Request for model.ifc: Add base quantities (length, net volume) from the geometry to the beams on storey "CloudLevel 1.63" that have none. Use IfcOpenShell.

First a look at what the model holds.

```python
import ifcopenshell
import ifcopenshell.util.element
import ifcopenshell.util.unit

model = ifcopenshell.open("model.ifc")
print(model.schema)
for unit_type in ("LENGTHUNIT", "AREAUNIT", "VOLUMEUNIT"):
    print(unit_type, ifcopenshell.util.unit.calculate_unit_scale(model, unit_type))
storey = next(s for s in model.by_type("IfcBuildingStorey") if s.Name == "CloudLevel 1.63")
beams = [e for e in ifcopenshell.util.element.get_decomposition(storey) if e.is_a("IfcBeam")]
for e in sorted(beams, key=lambda e: e.id()):
    print(e.id(), e.is_a(), e.Name, list(ifcopenshell.util.element.get_psets(e, qtos_only=True)), sep=" | ")
```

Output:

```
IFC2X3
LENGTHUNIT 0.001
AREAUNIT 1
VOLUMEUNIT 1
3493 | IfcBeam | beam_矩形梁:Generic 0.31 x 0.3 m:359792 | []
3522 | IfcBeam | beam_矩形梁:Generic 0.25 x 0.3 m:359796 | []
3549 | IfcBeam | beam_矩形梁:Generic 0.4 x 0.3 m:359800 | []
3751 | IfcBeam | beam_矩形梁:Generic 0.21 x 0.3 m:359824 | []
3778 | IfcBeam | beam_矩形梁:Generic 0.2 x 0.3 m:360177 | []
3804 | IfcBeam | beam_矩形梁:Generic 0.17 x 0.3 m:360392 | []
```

```python
import ifcopenshell
import ifcopenshell.api.pset
import ifcopenshell.geom
import ifcopenshell.util.element
import ifcopenshell.util.shape
import ifcopenshell.util.unit

model = ifcopenshell.open("model.ifc")
unit_scale = ifcopenshell.util.unit.calculate_unit_scale(model)
volume_scale = ifcopenshell.util.unit.calculate_unit_scale(model, "VOLUMEUNIT")
settings = ifcopenshell.geom.settings()

storey = next(s for s in model.by_type("IfcBuildingStorey") if s.Name == "CloudLevel 1.63")
beams = [e for e in ifcopenshell.util.element.get_decomposition(storey) if e.is_a("IfcBeam")]

for e in sorted(beams, key=lambda e: e.id()):
    if ifcopenshell.util.element.get_psets(e, qtos_only=True, should_inherit=False):
        continue
    # Geometry comes back in metres, in the element's own axes.
    shape = ifcopenshell.geom.create_shape(settings, e)
    values = {
        "Length": ifcopenshell.util.shape.get_max_xyz(shape.geometry) / unit_scale,
        "NetVolume": ifcopenshell.util.shape.get_volume(shape.geometry) / volume_scale,
    }
    qto = ifcopenshell.api.pset.add_qto(model, product=e, name="BaseQuantities")
    ifcopenshell.api.pset.edit_qto(model, qto=qto, properties=values)
    print(e.id(), {k: round(v, 3) for k, v in values.items()})

model.write("model_updated.ifc")
```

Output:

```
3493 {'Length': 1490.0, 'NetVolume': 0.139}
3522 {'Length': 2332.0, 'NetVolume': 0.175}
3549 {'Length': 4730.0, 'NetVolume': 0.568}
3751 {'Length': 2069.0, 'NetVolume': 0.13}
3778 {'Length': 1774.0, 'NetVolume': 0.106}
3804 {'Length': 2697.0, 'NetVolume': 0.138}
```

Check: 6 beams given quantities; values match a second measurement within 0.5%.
